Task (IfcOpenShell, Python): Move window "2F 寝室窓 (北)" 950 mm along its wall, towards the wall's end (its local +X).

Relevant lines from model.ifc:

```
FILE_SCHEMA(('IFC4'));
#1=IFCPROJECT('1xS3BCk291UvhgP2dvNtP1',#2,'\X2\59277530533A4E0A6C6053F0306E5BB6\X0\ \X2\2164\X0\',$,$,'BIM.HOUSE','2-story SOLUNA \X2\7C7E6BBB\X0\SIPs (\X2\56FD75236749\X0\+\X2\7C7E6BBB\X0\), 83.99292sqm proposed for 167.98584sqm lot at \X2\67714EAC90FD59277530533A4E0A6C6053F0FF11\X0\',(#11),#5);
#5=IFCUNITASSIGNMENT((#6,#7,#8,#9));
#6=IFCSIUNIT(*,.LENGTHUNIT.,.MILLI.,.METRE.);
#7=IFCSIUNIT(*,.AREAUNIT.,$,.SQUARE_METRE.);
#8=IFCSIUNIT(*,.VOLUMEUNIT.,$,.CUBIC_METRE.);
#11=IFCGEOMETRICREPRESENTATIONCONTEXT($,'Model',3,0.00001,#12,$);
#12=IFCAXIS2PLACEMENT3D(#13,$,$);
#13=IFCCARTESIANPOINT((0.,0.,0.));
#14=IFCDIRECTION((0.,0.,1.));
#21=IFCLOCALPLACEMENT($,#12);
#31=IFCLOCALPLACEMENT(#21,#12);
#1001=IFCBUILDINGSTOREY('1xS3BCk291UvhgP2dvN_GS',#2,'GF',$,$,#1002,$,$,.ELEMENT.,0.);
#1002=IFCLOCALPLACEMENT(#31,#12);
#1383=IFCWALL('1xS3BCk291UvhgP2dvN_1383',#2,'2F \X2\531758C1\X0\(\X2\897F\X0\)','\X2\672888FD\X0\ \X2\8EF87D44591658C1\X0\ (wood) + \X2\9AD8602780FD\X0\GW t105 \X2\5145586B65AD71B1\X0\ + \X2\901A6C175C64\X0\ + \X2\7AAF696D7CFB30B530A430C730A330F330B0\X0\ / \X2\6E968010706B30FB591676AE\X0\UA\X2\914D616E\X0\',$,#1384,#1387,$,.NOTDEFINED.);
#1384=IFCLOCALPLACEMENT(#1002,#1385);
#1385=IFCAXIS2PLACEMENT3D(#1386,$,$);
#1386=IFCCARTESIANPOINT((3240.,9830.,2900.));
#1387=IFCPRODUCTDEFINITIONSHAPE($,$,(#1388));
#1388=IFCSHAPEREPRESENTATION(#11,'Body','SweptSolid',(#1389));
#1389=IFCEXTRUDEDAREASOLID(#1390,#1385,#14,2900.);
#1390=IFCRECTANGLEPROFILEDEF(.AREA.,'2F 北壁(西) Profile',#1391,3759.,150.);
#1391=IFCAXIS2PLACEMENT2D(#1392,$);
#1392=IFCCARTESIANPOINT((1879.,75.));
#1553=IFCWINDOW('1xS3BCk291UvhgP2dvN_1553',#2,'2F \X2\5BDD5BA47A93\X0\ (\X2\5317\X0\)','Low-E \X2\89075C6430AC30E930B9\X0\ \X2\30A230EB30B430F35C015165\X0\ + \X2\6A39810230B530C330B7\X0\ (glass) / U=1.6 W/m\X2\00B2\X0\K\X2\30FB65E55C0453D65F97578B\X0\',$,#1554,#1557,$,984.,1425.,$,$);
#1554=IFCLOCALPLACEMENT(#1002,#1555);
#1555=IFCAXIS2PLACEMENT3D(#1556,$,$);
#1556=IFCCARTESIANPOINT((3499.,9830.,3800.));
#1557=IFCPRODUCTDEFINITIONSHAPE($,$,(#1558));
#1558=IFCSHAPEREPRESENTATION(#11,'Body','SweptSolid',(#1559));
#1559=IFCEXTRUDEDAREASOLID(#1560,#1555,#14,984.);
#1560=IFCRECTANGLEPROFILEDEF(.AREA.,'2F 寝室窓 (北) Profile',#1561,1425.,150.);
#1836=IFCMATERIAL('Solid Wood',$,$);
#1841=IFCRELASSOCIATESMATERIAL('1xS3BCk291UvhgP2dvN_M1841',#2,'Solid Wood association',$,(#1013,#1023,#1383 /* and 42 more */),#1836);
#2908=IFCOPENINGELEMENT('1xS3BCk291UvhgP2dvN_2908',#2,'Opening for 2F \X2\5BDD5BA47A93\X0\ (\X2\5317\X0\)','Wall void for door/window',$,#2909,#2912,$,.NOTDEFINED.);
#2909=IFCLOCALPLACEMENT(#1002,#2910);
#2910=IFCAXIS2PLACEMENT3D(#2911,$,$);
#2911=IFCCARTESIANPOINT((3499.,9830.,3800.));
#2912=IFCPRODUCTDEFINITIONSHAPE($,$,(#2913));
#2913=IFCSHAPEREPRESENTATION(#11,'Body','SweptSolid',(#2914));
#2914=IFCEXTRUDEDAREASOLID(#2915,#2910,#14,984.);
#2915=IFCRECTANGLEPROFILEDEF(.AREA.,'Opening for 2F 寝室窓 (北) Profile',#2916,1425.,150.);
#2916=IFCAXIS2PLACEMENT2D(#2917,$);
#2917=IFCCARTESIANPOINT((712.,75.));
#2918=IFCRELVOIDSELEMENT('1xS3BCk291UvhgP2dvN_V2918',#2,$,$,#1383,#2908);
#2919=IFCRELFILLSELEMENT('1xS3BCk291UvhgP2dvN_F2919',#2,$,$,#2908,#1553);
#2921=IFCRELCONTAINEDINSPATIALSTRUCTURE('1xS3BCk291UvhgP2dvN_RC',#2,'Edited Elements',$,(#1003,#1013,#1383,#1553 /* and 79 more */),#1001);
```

```python
import ifcopenshell
import ifcopenshell.api.geometry
import ifcopenshell.util.placement
import ifcopenshell.util.unit

model = ifcopenshell.open("model.ifc")
unit_scale = ifcopenshell.util.unit.calculate_unit_scale(model)

window = model.by_guid("1xS3BCk291UvhgP2dvN_1553")
opening = window.FillsVoids[0].RelatingOpeningElement
wall = opening.VoidsElements[0].RelatingBuildingElement

wall_matrix = ifcopenshell.util.placement.get_local_placement(wall.ObjectPlacement)
shift = wall_matrix[:3, 0] * 0.95 / unit_scale
before = ifcopenshell.util.placement.get_local_placement(window.ObjectPlacement)[:3, 3].copy()

# The window is not placed relative to its opening, so move both.
for product in (opening, window):
    matrix = ifcopenshell.util.placement.get_local_placement(product.ObjectPlacement)
    matrix[:3, 3] += shift
    ifcopenshell.api.geometry.edit_object_placement(model, product=product, matrix=matrix, is_si=False)

after = ifcopenshell.util.placement.get_local_placement(window.ObjectPlacement)[:3, 3]
print("window moved by", (after - before).round(3) + 0.0)

model.write("model_rev.ifc")
```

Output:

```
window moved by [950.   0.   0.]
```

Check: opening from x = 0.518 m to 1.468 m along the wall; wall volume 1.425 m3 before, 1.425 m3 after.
